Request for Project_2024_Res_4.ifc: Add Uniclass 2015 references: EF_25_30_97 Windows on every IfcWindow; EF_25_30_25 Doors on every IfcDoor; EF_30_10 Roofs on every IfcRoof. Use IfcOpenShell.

First a look at what the model holds.

```python
import ifcopenshell

model = ifcopenshell.open("Project_2024_Res_4.ifc")
print(model.schema)
print("classifications:", [c.Name for c in model.by_type("IfcClassification")])
for ifc_class in ("IfcDoor", "IfcRoof", "IfcStair", "IfcWall", "IfcWindow"):
    print(ifc_class, len(model.by_type(ifc_class)))
```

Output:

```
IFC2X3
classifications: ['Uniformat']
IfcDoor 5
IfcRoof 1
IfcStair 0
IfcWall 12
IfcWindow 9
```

```python
import ifcopenshell
import ifcopenshell.api.classification

model = ifcopenshell.open("Project_2024_Res_4.ifc")

# IFC2X3 requires Source and Edition and has no link from the project to the system.
system = model.create_entity("IfcClassification", Source="NBS", Edition="2015", Name="Uniclass 2015")

codes = {
    "IfcWindow": ("EF_25_30_97", "Windows"),
    "IfcDoor": ("EF_25_30_25", "Doors"),
    "IfcRoof": ("EF_30_10", "Roofs"),
}
for ifc_class, (code, name) in codes.items():
    products = model.by_type(ifc_class)
    ifcopenshell.api.classification.add_reference(
        model, products=products, classification=system, identification=code, name=name
    )
    print(code, len(products))

model.write("Project_2024_Res_4_updated.ifc")
```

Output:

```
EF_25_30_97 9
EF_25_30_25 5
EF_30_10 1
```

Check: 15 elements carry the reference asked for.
